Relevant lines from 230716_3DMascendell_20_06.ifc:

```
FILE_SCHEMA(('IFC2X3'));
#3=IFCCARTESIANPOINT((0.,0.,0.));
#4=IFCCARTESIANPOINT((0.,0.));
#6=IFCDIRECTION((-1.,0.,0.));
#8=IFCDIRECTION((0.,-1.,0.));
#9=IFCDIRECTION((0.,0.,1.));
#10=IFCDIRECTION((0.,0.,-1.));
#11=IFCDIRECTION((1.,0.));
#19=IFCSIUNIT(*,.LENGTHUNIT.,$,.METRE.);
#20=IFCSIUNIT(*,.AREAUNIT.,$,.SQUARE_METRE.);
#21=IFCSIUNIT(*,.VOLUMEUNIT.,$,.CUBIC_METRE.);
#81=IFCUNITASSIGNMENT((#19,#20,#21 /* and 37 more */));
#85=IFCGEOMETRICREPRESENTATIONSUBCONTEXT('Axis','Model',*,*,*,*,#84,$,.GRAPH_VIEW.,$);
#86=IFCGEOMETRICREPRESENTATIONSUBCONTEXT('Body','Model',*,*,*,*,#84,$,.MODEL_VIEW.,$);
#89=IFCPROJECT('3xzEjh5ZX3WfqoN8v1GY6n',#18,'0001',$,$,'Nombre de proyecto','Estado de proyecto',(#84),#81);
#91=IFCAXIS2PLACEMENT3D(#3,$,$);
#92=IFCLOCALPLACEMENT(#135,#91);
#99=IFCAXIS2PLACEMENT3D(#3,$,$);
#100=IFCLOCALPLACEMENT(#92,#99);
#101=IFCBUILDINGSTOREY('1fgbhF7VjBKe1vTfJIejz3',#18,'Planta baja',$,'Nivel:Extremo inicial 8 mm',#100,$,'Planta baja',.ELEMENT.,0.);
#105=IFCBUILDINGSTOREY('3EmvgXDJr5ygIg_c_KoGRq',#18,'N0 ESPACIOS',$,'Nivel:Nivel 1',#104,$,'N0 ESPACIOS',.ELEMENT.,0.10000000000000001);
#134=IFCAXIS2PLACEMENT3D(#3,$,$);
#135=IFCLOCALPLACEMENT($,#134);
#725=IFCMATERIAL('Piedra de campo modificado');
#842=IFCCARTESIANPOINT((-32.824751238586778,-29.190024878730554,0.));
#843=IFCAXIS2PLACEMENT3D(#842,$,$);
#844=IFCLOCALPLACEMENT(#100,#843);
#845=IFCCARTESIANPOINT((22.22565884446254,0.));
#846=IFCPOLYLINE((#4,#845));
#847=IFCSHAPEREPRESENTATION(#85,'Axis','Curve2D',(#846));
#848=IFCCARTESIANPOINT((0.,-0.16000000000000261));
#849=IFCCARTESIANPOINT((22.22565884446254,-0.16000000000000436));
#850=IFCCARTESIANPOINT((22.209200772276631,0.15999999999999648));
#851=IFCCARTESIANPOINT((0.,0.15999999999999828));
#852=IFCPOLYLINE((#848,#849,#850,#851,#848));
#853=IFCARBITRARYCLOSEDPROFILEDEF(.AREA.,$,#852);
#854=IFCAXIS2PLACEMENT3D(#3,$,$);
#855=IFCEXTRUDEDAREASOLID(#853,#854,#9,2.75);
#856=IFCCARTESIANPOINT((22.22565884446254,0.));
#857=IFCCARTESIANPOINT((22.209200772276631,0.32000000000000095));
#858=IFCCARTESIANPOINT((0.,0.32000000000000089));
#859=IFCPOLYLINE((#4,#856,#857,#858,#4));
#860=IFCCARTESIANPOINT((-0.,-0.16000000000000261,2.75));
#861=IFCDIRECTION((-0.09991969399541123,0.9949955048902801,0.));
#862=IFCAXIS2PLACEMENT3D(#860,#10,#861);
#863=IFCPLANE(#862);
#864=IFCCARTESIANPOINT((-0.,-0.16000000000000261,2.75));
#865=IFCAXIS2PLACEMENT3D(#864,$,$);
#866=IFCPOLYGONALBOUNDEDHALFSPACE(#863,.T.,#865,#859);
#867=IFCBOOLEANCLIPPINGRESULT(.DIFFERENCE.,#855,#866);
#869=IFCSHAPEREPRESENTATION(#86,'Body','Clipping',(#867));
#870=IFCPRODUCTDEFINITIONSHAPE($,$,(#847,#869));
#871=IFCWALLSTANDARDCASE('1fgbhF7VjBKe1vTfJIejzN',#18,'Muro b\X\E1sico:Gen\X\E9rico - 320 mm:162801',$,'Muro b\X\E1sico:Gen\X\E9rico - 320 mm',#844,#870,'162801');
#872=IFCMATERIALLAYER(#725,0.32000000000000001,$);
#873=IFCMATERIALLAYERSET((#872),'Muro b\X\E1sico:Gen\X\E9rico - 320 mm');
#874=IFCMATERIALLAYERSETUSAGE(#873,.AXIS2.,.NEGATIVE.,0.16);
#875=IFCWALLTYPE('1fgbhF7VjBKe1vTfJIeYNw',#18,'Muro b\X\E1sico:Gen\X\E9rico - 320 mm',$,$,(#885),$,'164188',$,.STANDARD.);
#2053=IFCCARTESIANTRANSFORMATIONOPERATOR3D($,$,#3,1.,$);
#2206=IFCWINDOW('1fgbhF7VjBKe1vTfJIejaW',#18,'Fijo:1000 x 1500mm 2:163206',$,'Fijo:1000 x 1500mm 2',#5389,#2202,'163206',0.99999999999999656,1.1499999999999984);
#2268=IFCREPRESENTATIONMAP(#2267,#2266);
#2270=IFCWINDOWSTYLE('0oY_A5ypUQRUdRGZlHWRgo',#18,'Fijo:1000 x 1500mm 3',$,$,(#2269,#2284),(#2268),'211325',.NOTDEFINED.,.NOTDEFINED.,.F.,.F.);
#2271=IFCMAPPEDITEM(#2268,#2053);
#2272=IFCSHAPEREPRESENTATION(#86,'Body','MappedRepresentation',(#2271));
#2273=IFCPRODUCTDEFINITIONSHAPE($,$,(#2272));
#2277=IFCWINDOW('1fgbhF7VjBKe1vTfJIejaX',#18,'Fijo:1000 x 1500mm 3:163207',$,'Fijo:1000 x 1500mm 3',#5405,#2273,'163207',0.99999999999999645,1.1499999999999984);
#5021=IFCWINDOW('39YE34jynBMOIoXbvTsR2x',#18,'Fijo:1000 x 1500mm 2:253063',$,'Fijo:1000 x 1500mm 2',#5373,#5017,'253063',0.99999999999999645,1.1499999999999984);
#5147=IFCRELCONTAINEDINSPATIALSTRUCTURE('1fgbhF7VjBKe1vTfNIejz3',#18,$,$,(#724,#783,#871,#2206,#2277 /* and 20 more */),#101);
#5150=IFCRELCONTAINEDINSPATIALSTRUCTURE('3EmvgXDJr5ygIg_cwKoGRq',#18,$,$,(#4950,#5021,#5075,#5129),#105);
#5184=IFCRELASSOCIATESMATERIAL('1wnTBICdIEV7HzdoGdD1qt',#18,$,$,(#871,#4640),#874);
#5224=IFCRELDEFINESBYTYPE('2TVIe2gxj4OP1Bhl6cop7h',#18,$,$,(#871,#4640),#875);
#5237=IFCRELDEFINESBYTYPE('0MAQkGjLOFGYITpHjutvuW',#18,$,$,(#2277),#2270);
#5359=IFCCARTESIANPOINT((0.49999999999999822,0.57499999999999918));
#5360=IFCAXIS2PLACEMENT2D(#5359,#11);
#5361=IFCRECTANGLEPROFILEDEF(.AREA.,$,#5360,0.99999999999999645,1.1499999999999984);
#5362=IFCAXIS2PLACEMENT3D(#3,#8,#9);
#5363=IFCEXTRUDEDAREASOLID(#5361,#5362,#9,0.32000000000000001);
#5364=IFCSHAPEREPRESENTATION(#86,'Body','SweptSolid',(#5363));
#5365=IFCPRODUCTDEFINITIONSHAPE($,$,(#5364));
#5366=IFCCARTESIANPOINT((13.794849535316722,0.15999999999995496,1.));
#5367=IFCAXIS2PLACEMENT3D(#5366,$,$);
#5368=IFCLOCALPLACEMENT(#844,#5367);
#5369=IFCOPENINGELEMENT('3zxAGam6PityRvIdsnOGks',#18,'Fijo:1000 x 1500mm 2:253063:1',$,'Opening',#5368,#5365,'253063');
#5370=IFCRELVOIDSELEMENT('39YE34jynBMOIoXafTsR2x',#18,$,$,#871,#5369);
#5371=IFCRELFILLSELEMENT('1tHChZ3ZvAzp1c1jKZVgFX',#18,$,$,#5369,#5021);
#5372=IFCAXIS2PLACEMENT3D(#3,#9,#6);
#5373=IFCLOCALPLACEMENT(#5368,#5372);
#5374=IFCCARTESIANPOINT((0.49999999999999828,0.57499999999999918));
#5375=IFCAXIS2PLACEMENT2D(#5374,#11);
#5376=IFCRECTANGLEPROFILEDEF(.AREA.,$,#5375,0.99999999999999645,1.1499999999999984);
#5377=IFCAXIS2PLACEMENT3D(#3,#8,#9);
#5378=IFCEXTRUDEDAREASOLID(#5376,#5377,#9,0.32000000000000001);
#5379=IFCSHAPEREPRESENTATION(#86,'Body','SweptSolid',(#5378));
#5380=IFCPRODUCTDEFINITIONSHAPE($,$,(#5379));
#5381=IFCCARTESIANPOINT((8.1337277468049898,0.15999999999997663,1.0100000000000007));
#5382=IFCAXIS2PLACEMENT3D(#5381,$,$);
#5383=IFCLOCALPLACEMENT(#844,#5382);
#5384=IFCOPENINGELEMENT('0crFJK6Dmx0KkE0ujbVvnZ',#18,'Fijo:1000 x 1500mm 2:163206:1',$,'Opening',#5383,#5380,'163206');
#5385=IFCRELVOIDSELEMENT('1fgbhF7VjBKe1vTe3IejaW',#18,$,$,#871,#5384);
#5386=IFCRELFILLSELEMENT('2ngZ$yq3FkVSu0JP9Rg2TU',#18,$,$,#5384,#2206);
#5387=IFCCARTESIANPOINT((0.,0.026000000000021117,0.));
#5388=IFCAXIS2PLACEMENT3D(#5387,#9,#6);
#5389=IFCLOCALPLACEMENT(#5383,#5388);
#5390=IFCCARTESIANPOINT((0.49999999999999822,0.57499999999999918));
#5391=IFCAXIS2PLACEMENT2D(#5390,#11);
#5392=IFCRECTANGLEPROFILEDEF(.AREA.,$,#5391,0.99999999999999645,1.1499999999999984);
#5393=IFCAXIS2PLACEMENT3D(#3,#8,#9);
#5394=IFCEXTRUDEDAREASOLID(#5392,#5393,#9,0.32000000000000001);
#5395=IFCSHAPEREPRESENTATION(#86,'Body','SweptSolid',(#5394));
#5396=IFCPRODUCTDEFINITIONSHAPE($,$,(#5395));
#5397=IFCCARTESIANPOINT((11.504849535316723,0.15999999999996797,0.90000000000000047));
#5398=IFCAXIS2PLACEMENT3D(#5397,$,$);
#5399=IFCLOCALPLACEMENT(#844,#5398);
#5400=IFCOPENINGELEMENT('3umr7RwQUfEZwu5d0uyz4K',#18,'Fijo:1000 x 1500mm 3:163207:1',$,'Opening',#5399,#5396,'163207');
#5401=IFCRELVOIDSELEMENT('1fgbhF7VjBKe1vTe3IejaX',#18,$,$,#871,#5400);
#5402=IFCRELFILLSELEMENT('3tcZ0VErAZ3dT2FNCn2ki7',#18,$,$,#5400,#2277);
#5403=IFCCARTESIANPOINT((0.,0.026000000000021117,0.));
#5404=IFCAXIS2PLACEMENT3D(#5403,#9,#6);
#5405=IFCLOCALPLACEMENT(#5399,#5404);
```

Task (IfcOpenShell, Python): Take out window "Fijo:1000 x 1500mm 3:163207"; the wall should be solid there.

```python
import ifcopenshell
import ifcopenshell.api.feature
import ifcopenshell.api.root
import ifcopenshell.geom
import ifcopenshell.util.shape

model = ifcopenshell.open("230716_3DMascendell_20_06.ifc")
settings = ifcopenshell.geom.settings()


def volume(element):
    """Net volume in cubic metres, openings subtracted."""
    shape = ifcopenshell.geom.create_shape(settings, element)
    return ifcopenshell.util.shape.get_volume(shape.geometry)


window = model.by_id(2277)
opening = window.FillsVoids[0].RelatingOpeningElement
wall = opening.VoidsElements[0].RelatingBuildingElement
before = volume(wall)

ifcopenshell.api.root.remove_product(model, product=window)
ifcopenshell.api.feature.remove_feature(model, feature=opening)

after = volume(wall)

print(f"wall volume {before:.3f} -> {after:.3f} m3")

model.write("230716_3DMascendell_20_06_updated.ifc")
```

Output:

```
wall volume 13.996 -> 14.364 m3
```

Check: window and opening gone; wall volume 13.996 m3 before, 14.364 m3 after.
